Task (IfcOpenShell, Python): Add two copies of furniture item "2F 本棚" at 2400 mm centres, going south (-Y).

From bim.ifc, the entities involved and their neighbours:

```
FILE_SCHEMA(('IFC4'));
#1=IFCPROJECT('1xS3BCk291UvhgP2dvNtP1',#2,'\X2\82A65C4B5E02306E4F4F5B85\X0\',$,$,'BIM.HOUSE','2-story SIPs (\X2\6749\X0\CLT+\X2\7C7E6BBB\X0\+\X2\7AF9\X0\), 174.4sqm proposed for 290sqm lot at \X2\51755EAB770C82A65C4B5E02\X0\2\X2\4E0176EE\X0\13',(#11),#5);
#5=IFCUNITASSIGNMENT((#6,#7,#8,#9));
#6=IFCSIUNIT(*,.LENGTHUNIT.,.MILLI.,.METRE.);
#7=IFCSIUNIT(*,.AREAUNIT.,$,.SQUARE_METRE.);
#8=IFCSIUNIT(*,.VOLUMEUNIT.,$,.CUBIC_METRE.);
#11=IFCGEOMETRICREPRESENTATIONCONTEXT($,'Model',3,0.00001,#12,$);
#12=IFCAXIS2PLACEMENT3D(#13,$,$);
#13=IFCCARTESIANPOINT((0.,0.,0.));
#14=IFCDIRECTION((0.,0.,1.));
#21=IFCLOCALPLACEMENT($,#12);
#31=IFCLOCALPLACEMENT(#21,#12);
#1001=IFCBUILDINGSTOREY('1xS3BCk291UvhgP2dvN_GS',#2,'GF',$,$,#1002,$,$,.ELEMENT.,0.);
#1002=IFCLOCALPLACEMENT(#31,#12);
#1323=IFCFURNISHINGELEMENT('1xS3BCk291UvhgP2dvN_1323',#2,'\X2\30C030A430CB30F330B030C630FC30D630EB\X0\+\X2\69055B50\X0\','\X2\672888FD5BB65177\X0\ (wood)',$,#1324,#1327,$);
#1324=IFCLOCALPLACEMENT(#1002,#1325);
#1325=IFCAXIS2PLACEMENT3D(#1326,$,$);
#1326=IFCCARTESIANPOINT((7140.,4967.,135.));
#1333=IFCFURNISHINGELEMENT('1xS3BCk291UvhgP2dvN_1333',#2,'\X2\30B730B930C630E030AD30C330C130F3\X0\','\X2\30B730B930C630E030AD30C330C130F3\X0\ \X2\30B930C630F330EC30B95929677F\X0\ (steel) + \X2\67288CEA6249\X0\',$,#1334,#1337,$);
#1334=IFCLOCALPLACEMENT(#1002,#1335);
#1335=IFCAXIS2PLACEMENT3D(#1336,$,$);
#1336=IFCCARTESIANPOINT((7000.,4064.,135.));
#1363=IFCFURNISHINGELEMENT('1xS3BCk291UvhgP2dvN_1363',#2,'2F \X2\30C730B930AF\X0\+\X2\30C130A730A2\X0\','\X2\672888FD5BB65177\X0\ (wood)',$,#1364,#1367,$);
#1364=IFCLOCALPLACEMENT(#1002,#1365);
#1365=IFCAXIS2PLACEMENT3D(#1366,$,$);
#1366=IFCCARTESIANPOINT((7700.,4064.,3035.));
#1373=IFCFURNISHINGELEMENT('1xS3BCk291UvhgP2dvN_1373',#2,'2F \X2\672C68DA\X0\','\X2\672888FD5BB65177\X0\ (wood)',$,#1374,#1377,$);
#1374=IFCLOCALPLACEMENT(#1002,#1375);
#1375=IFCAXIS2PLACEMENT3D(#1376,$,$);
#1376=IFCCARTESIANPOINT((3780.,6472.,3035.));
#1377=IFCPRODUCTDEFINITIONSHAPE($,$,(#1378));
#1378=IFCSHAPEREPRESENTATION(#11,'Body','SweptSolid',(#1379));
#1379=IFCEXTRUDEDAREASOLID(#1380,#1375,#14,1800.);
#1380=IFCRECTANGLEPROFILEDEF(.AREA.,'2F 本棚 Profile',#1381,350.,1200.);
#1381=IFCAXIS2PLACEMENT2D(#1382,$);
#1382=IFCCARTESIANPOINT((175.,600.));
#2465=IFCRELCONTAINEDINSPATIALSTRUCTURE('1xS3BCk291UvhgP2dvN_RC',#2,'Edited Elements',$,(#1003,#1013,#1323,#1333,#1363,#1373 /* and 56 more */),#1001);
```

```python
import numpy as np
import ifcopenshell
import ifcopenshell.api.geometry
import ifcopenshell.api.root
import ifcopenshell.util.element
import ifcopenshell.util.placement

model = ifcopenshell.open("bim.ifc")


def reuse_history(source, copy):
    """copy_class also copies each property set's owner history, people and application; keep the originals."""
    for rel in copy.IsDefinedBy:
        if rel.is_a("IfcRelDefinesByProperties") and (history := rel.RelatingPropertyDefinition.OwnerHistory):
            rel.RelatingPropertyDefinition.OwnerHistory = source.OwnerHistory
            ifcopenshell.util.element.remove_deep2(model, history)


source = model.by_guid("1xS3BCk291UvhgP2dvN_1373")
base = ifcopenshell.util.placement.get_local_placement(source.ObjectPlacement)
step = np.array([0.0, -1.0, 0.0]) * 2400.0

for i in range(1, 3):
    copy = ifcopenshell.api.root.copy_class(model, product=source)
    copy.Representation = ifcopenshell.util.element.copy_deep(
        model, source.Representation, exclude=["IfcGeometricRepresentationContext", "IfcRepresentationMap"]
    )
    reuse_history(source, copy)
    matrix = base.copy()
    matrix[:3, 3] += i * step
    print("added at", matrix[:3, 3].round(3) + 0.0)
    ifcopenshell.api.geometry.edit_object_placement(model, product=copy, matrix=matrix, is_si=False)

model.write("bim-out.ifc")
```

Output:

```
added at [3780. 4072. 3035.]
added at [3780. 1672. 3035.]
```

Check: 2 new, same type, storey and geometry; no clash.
